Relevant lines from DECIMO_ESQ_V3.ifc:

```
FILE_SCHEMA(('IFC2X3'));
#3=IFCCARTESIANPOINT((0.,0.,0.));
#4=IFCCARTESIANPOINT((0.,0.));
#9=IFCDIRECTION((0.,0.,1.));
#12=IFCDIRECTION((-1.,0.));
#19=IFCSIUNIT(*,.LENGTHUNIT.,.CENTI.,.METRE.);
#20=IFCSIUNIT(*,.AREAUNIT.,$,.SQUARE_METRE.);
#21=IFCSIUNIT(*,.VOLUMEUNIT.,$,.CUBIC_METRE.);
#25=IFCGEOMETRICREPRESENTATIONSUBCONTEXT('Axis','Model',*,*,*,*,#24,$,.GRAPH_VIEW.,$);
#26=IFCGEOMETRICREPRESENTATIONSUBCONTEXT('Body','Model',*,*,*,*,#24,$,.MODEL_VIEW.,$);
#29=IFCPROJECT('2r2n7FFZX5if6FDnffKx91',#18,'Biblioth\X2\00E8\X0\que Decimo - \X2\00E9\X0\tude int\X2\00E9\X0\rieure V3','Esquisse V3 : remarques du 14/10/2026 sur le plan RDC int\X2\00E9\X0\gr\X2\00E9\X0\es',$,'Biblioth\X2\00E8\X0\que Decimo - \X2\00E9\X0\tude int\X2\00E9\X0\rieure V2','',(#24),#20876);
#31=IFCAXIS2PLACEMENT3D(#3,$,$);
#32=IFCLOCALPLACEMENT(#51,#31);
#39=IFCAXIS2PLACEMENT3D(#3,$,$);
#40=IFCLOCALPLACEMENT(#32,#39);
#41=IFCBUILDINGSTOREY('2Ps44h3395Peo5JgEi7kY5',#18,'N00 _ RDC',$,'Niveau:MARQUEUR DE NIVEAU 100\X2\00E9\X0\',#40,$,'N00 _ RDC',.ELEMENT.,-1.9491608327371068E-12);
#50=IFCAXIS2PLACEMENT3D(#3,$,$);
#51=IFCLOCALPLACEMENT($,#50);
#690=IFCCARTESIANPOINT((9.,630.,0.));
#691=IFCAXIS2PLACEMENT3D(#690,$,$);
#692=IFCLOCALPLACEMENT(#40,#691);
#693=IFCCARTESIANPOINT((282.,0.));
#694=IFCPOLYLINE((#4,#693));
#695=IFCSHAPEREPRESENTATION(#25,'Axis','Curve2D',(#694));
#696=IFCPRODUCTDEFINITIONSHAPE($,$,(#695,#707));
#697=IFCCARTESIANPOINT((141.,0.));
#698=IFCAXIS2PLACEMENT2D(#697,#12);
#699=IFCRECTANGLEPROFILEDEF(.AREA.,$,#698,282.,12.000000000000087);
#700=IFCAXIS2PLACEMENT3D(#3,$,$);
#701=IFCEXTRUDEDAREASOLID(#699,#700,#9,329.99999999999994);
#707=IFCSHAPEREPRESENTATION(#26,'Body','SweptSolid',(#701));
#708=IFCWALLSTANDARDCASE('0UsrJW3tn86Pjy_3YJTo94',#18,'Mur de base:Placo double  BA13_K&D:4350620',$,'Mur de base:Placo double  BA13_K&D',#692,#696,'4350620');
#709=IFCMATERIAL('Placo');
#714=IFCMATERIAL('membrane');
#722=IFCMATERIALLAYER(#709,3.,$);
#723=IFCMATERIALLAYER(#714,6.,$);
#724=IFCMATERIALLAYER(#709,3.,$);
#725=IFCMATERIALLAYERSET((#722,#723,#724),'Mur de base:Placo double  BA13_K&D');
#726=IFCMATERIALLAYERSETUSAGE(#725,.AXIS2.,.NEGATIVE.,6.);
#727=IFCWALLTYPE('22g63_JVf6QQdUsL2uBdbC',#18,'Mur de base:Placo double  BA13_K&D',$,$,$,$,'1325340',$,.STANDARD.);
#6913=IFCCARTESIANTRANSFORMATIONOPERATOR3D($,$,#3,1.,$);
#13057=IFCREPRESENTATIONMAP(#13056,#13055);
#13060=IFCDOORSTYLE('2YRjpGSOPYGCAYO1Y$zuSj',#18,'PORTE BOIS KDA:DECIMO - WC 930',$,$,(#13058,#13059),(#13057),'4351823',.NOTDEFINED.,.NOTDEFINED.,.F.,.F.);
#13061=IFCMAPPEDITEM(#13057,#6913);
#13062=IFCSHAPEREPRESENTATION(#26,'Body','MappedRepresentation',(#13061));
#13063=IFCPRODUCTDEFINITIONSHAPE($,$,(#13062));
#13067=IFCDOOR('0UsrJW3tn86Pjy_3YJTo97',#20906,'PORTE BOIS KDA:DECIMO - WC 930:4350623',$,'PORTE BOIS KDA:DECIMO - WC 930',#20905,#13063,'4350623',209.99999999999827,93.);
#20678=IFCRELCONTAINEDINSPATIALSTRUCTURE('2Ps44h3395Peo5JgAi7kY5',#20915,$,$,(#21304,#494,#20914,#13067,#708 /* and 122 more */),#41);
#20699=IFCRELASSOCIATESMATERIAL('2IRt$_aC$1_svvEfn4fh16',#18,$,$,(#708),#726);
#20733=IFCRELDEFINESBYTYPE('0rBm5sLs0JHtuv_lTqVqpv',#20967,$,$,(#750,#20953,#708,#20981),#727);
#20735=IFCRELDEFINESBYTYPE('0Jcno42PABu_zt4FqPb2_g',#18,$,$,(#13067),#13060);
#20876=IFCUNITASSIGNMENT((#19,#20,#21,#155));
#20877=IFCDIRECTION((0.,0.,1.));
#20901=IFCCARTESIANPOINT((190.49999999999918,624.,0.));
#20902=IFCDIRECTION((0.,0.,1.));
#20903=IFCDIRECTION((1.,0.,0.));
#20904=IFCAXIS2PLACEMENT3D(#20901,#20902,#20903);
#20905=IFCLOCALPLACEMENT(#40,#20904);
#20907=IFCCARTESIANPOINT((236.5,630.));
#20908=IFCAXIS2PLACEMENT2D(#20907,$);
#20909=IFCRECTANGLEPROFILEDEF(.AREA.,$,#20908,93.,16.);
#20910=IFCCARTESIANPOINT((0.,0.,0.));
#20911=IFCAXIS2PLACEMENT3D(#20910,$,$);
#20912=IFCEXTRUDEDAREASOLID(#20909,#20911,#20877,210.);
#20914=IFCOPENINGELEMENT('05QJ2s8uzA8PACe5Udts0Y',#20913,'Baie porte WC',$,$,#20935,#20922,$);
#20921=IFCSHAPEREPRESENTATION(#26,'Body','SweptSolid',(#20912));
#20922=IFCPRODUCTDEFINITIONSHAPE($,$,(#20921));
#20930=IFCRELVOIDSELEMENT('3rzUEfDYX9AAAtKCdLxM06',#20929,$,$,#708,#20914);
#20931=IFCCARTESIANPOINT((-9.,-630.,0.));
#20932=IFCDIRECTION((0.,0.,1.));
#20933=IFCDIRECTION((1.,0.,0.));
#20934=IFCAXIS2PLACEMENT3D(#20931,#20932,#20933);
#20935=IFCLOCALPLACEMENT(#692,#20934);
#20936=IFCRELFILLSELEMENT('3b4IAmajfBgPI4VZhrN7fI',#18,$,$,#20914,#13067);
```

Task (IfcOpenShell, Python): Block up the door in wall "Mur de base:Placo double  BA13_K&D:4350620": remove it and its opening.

```python
import ifcopenshell
import ifcopenshell.api.feature
import ifcopenshell.api.root
import ifcopenshell.geom
import ifcopenshell.util.shape

model = ifcopenshell.open("DECIMO_ESQ_V3.ifc")
settings = ifcopenshell.geom.settings()


def volume(element):
    """Net volume in cubic metres, openings subtracted."""
    shape = ifcopenshell.geom.create_shape(settings, element)
    return ifcopenshell.util.shape.get_volume(shape.geometry)


door = model.by_guid("0UsrJW3tn86Pjy_3YJTo97")
opening = door.FillsVoids[0].RelatingOpeningElement
wall = opening.VoidsElements[0].RelatingBuildingElement
before = volume(wall)

ifcopenshell.api.root.remove_product(model, product=door)
ifcopenshell.api.feature.remove_feature(model, feature=opening)

after = volume(wall)

print(f"wall volume {before:.3f} -> {after:.3f} m3")

model.write("DECIMO_ESQ_V3_rev.ifc")
```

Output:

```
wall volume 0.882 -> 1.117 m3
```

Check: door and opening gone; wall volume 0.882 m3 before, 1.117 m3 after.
